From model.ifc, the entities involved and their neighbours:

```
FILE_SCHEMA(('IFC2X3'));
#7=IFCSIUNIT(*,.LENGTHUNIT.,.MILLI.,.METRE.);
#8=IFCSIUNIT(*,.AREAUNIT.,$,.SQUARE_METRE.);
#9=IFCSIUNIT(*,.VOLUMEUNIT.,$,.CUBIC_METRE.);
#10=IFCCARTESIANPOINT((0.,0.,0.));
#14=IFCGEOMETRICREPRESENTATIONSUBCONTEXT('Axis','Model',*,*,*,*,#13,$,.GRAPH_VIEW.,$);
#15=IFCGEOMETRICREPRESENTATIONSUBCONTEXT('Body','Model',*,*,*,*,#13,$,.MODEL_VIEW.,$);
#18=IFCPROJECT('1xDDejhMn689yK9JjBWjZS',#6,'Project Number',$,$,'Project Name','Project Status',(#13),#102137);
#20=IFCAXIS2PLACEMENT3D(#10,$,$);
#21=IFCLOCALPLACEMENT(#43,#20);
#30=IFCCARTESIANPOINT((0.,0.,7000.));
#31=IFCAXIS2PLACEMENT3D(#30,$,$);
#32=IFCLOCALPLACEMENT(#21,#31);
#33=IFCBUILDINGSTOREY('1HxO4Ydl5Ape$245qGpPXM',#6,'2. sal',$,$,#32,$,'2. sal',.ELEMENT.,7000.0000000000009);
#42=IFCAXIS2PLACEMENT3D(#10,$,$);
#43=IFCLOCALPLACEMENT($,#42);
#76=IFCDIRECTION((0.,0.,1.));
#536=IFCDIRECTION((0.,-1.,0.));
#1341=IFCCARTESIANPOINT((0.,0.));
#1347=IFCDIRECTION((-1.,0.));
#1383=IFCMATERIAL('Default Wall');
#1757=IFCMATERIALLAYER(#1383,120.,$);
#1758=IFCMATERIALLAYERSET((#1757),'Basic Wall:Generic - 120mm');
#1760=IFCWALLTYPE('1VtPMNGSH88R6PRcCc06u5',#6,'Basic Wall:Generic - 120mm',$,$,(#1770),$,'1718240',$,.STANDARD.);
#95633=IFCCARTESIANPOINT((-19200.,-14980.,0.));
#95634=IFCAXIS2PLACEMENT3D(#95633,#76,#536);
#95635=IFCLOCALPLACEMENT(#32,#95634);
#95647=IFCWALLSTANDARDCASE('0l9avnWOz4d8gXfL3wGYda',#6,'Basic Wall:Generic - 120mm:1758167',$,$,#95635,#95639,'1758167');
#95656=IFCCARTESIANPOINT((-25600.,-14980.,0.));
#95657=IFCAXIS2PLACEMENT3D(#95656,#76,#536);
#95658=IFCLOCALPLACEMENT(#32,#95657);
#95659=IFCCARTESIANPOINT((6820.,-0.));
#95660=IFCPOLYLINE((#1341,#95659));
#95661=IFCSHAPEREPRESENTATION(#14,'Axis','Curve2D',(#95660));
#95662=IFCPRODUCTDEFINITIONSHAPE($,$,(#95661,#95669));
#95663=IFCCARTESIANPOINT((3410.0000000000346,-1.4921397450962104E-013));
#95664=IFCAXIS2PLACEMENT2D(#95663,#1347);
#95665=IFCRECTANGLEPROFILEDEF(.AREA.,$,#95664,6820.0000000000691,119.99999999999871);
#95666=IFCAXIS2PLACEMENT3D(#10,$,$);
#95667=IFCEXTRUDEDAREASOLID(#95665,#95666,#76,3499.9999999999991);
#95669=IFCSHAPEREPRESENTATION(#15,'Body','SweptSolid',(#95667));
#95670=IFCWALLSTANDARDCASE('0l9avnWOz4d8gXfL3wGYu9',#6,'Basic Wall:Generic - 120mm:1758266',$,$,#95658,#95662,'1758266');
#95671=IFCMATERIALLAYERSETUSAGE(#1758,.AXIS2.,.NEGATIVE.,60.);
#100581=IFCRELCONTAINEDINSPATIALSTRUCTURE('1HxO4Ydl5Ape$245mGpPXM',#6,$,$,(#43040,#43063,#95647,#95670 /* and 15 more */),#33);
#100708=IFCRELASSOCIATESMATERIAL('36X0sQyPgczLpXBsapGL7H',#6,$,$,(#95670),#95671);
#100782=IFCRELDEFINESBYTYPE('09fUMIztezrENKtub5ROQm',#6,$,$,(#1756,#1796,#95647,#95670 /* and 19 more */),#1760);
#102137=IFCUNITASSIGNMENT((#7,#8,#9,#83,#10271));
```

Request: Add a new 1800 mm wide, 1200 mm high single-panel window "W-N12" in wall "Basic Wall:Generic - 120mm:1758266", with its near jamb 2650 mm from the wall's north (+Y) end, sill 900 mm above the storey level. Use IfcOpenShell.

```python
import numpy as np
import ifcopenshell
import ifcopenshell.api.feature
import ifcopenshell.api.geometry
import ifcopenshell.api.root
import ifcopenshell.api.spatial
import ifcopenshell.api.type
import ifcopenshell.geom
import ifcopenshell.util.element
import ifcopenshell.util.placement
import ifcopenshell.util.representation
import ifcopenshell.util.shape
import ifcopenshell.util.unit

model = ifcopenshell.open("model.ifc")
unit_scale = ifcopenshell.util.unit.calculate_unit_scale(model)
settings = ifcopenshell.geom.settings()


def volume(element):
    """Net volume in cubic metres, openings subtracted."""
    shape = ifcopenshell.geom.create_shape(settings, element)
    return ifcopenshell.util.shape.get_volume(shape.geometry)


wall = model.by_id(95670)
storey = ifcopenshell.util.element.get_container(wall, ifc_class="IfcBuildingStorey")
context = ifcopenshell.util.representation.get_context(model, "Model", "Body", "MODEL_VIEW")
before = volume(wall)

width, height, from_end, sill = 1.8, 1.2, 2.65, 0.9  # metres

# The wall runs along its own X axis, and the end named is its -X end.
wall_shape = ifcopenshell.geom.create_shape(settings, wall)
x, y, z = ifcopenshell.util.shape.get_vertices(wall_shape.geometry).T
start = x.min() + from_end
face, thickness = float(y.min()), float(y.max() - y.min())
wall_matrix = ifcopenshell.util.placement.get_local_placement(wall.ObjectPlacement)
level = ifcopenshell.util.placement.get_local_placement(storey.ObjectPlacement)[2, 3]


def in_wall(x, y):
    """Placement at x, y metres in the wall's axes, at sill height."""
    matrix = wall_matrix.copy()
    matrix[:, 3] = wall_matrix @ np.array([x / unit_scale, y / unit_scale, 0.0, 1.0])
    matrix[2, 3] = level + sill / unit_scale
    return matrix


# Opening: a box that overshoots both wall faces by 50 mm.
opening = ifcopenshell.api.root.create_entity(model, ifc_class="IfcOpeningElement")
box = ifcopenshell.api.geometry.add_wall_representation(
    model, context=context, length=width, height=height, thickness=thickness + 0.1
)
ifcopenshell.api.geometry.assign_representation(model, product=opening, representation=box)
ifcopenshell.api.geometry.edit_object_placement(model, product=opening, matrix=in_wall(start, face - 0.05), is_si=False)
ifcopenshell.api.feature.add_feature(model, feature=opening, element=wall)

window = ifcopenshell.api.root.create_entity(model, ifc_class="IfcWindow", name="W-N12")
window.OverallWidth, window.OverallHeight = width / unit_scale, height / unit_scale
body = ifcopenshell.api.geometry.add_window_representation(
    model,
    context=context,
    overall_width=window.OverallWidth,
    overall_height=window.OverallHeight,
    partition_type="SINGLE_PANEL",
)
ifcopenshell.api.geometry.assign_representation(model, product=window, representation=body)
ifcopenshell.api.spatial.assign_container(model, products=[window], relating_structure=storey)
fills = ifcopenshell.api.feature.add_filling(model, opening=opening, element=window)
fills.OwnerHistory = window.OwnerHistory  # required in IFC2X3

# IFC2X3 keeps the operation on the window style.
style = ifcopenshell.api.root.create_entity(model, ifc_class="IfcWindowStyle", name="W-N12")
style.OperationType, style.ConstructionType = "SINGLE_PANEL", "NOTDEFINED"
style.ParameterTakesPrecedence = style.Sizeable = False
ifcopenshell.api.type.assign_type(model, related_objects=[window], relating_type=style)

# Centre the window in the wall's thickness.
ifcopenshell.api.geometry.edit_object_placement(model, product=window, matrix=in_wall(start, face), is_si=False)
window_shape = ifcopenshell.geom.create_shape(settings, window)
depth = ifcopenshell.util.shape.get_vertices(window_shape.geometry)[:, 1]
offset = face + thickness / 2 - (depth.min() + depth.max()) / 2
ifcopenshell.api.geometry.edit_object_placement(model, product=window, matrix=in_wall(start, offset), is_si=False)

after = volume(wall)

print(f"wall volume {before:.3f} -> {after:.3f} m3")

model.write("model_v2.ifc")
```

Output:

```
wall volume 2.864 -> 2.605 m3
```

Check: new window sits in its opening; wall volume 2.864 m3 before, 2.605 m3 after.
